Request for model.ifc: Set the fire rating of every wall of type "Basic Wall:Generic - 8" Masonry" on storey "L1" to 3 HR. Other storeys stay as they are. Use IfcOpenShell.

First a look at what the model holds.

```python
import ifcopenshell
import ifcopenshell.util.element

model = ifcopenshell.open("model.ifc")
print(model.schema)
storey = next(s for s in model.by_type("IfcBuildingStorey") if s.Name == "L1")
walls = [e for e in ifcopenshell.util.element.get_decomposition(storey) if e.is_a("IfcWall")]
seen = {}
for e in walls:
    element_type = ifcopenshell.util.element.get_type(e)
    key = (element_type.Name if element_type != e and element_type else None, ifcopenshell.util.element.get_pset(e, "Pset_WallCommon", "FireRating"))
    seen[key] = seen.get(key, 0) + 1
for (name, value), count in sorted(seen.items(), key=str):
    print(count, "x", name, "|", value)
```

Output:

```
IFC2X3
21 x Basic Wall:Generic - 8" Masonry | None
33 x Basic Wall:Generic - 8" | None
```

```python
import ifcopenshell
import ifcopenshell.api.pset
import ifcopenshell.util.element

model = ifcopenshell.open("model.ifc")

storey = next(s for s in model.by_type("IfcBuildingStorey") if s.Name == "L1")
walls = [e for e in ifcopenshell.util.element.get_decomposition(storey) if e.is_a("IfcWall")]

count = 0
for e in walls:
    element_type = ifcopenshell.util.element.get_type(e)
    if element_type in (None, e) or element_type.Name != 'Basic Wall:Generic - 8" Masonry':
        continue
    # add_pset returns the element's existing set when there is one.
    pset = ifcopenshell.api.pset.add_pset(model, product=e, name="Pset_WallCommon")
    ifcopenshell.api.pset.edit_pset(model, pset=pset, properties={"FireRating": "3 HR"})
    count += 1

print(count, "walls updated")

model.write("model_v2.ifc")
```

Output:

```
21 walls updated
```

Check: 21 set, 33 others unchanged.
